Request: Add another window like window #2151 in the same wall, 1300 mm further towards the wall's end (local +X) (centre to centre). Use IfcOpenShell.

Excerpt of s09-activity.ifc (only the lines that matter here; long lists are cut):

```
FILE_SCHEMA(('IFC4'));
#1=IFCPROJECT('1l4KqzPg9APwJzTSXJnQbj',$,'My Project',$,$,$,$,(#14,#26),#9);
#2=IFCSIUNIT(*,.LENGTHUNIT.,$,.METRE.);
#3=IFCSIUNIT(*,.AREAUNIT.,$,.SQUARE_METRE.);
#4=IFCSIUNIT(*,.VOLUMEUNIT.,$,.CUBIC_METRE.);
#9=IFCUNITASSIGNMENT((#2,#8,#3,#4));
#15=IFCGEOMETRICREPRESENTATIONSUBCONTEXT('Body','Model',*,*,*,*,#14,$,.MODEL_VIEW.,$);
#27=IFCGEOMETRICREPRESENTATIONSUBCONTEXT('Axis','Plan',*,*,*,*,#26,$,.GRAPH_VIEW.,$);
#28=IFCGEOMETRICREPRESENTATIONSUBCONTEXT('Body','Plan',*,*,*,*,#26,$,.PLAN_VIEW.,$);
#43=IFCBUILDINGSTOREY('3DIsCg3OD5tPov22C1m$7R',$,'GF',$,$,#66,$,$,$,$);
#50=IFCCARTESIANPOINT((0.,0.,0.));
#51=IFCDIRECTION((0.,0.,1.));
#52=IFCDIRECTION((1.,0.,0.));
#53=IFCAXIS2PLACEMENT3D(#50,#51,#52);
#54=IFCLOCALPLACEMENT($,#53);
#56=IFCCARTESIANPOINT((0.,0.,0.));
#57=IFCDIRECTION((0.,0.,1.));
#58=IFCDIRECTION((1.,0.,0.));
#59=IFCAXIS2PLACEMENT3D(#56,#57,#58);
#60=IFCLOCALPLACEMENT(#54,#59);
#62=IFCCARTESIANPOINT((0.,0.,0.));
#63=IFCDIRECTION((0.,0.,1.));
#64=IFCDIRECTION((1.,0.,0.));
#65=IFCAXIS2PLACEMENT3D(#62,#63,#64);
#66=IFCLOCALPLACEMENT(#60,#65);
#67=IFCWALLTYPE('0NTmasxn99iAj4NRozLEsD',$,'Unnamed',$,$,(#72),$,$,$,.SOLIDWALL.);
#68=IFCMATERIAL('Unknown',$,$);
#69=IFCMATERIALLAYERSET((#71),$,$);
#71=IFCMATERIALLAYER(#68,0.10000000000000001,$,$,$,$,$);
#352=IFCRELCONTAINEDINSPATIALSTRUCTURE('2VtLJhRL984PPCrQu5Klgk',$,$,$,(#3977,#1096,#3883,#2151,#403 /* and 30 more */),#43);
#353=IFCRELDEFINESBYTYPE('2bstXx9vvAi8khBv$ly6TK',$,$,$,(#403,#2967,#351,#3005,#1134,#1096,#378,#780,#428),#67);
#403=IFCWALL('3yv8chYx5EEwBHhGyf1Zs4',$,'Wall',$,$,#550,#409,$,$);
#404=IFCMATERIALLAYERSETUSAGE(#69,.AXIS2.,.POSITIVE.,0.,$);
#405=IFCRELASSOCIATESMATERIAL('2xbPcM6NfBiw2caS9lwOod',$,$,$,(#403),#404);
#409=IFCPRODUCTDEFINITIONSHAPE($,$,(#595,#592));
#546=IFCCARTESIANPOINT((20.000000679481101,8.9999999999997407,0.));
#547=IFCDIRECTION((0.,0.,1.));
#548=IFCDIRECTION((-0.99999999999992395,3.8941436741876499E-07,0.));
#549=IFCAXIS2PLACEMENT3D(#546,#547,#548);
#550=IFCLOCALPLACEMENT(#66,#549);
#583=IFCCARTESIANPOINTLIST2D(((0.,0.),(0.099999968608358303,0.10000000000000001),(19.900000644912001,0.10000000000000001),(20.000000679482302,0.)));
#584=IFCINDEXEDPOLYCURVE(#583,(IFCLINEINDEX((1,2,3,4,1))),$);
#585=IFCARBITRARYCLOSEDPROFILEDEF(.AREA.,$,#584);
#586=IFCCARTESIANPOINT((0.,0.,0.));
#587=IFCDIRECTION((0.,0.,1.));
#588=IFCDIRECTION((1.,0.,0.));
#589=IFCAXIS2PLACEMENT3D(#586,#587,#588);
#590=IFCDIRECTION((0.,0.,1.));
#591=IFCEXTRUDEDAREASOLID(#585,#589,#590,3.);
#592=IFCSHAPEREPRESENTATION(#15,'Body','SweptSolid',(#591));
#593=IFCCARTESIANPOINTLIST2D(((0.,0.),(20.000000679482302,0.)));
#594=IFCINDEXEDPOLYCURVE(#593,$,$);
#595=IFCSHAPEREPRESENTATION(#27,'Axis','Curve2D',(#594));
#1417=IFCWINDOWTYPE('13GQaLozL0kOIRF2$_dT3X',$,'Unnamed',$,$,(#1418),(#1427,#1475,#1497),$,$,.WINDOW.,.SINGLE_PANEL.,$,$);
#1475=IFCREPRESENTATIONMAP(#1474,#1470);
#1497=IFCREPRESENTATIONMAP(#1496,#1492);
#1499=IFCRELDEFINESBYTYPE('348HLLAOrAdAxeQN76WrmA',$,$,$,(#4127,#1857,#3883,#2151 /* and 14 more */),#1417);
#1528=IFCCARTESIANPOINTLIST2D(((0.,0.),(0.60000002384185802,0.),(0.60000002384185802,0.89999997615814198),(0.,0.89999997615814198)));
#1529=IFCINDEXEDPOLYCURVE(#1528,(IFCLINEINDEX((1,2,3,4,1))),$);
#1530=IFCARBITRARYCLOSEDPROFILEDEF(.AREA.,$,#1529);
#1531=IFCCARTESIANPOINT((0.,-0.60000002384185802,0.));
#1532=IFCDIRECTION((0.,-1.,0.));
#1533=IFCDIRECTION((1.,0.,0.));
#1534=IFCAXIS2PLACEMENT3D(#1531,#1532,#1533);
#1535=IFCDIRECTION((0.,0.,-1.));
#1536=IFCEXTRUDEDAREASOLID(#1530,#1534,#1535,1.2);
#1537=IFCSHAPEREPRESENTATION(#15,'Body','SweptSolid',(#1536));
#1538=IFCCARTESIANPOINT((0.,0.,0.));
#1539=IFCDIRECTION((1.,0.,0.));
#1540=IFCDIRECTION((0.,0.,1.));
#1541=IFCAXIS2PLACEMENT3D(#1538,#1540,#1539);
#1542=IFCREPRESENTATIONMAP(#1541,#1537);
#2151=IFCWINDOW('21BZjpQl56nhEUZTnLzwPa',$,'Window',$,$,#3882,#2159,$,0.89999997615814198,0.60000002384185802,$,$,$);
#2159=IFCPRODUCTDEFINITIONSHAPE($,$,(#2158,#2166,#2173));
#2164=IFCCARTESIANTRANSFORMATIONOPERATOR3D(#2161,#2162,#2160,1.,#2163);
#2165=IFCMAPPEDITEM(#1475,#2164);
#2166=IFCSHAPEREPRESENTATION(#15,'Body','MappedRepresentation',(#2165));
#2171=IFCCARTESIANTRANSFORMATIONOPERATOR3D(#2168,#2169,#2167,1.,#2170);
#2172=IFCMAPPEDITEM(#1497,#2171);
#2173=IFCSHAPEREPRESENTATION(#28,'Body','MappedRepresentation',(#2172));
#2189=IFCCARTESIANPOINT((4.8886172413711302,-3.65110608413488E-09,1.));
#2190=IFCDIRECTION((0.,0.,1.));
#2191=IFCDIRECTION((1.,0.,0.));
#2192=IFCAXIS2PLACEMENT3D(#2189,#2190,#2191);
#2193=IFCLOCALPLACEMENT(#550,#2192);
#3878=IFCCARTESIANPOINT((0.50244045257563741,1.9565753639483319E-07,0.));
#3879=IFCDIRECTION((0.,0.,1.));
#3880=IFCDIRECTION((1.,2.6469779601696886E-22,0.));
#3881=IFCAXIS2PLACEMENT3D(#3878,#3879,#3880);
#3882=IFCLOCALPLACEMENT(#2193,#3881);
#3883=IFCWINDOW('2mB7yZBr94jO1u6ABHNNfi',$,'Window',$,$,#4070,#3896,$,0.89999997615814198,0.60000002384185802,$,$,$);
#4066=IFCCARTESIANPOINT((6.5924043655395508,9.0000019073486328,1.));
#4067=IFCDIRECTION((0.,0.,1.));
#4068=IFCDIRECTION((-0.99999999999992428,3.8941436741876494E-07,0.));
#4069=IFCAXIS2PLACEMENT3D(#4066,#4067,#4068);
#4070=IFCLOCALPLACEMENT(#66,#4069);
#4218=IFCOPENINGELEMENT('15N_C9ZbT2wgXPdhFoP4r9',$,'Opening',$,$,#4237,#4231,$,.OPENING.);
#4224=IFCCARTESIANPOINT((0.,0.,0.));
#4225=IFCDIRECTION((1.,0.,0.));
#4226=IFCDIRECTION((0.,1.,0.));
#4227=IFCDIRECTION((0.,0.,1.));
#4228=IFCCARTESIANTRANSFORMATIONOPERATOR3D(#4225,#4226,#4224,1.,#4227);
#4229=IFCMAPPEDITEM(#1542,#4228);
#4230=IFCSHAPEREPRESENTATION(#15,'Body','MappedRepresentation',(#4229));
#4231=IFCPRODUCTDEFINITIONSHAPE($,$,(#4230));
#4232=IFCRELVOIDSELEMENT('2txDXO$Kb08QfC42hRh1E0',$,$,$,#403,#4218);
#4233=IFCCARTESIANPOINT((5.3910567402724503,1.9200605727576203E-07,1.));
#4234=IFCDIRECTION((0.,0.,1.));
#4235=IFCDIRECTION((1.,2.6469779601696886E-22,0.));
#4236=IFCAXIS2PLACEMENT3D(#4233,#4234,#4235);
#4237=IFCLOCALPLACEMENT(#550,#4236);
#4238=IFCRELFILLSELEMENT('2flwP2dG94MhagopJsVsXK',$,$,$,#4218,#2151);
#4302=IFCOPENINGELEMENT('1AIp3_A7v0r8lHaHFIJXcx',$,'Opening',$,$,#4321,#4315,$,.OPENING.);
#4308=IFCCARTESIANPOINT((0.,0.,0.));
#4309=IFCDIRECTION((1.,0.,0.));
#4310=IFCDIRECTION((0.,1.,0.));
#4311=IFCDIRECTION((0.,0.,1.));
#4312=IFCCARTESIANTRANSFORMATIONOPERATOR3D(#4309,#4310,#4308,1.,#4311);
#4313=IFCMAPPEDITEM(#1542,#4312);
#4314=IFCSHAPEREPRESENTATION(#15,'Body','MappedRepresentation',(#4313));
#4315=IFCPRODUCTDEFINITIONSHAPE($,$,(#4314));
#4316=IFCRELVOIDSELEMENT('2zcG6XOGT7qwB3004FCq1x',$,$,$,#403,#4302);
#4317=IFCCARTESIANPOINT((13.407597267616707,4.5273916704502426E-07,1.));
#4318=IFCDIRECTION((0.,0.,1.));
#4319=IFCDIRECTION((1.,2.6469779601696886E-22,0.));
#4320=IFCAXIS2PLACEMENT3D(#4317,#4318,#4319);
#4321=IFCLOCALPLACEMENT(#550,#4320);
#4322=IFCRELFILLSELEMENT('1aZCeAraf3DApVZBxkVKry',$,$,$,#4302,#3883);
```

```python
import ifcopenshell
import ifcopenshell.api.feature
import ifcopenshell.api.geometry
import ifcopenshell.api.root
import ifcopenshell.geom
import ifcopenshell.util.element
import ifcopenshell.util.placement
import ifcopenshell.util.shape

model = ifcopenshell.open("s09-activity.ifc")
settings = ifcopenshell.geom.settings()


def volume(element):
    """Net volume in cubic metres, openings subtracted."""
    shape = ifcopenshell.geom.create_shape(settings, element)
    return ifcopenshell.util.shape.get_volume(shape.geometry)


window = model.by_id(2151)
opening = window.FillsVoids[0].RelatingOpeningElement
wall = opening.VoidsElements[0].RelatingBuildingElement
before = volume(wall)
shift = ifcopenshell.util.placement.get_local_placement(wall.ObjectPlacement)[:3, 0] * 1.3

# copy_class copies the void relationship, type, container and properties, but no geometry.
new_opening = ifcopenshell.api.root.copy_class(model, product=opening)
new_opening.Representation = ifcopenshell.util.element.copy_deep(
    model, opening.Representation, exclude=["IfcGeometricRepresentationContext", "IfcRepresentationMap"]
)
new_window = ifcopenshell.api.root.copy_class(model, product=window)
new_window.Representation = ifcopenshell.util.element.copy_deep(
    model, window.Representation, exclude=["IfcGeometricRepresentationContext", "IfcRepresentationMap"]
)
ifcopenshell.api.feature.add_filling(model, opening=new_opening, element=new_window)

for old, new in ((opening, new_opening), (window, new_window)):
    matrix = ifcopenshell.util.placement.get_local_placement(old.ObjectPlacement)
    matrix[:3, 3] += shift
    ifcopenshell.api.geometry.edit_object_placement(model, product=new, matrix=matrix, is_si=False)

after = volume(wall)

print(f"wall volume {before:.3f} -> {after:.3f} m3")

model.write("s09-activity_v2.ifc")
```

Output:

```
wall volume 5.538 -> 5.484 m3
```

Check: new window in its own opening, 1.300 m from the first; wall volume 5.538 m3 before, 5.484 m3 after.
